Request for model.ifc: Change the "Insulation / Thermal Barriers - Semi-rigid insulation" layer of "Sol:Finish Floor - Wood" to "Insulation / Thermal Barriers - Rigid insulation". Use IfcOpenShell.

First a look at what the model holds.

```python
import ifcopenshell
import ifcopenshell.util.element

model = ifcopenshell.open("model.ifc")
print(model.schema)
for layer_set in model.by_type("IfcMaterialLayerSet"):
    if layer_set.LayerSetName == "Sol:Finish Floor - Wood":
        for layer in layer_set.MaterialLayers:
            print(layer.id(), layer.Material and layer.Material.Name, layer.LayerThickness, sep=" | ")
        print(len(ifcopenshell.util.element.get_elements_by_material(model, layer_set)), "elements and types use it")
print(sorted(m.Name for m in model.by_type("IfcMaterial") if m.Name)[:60])
```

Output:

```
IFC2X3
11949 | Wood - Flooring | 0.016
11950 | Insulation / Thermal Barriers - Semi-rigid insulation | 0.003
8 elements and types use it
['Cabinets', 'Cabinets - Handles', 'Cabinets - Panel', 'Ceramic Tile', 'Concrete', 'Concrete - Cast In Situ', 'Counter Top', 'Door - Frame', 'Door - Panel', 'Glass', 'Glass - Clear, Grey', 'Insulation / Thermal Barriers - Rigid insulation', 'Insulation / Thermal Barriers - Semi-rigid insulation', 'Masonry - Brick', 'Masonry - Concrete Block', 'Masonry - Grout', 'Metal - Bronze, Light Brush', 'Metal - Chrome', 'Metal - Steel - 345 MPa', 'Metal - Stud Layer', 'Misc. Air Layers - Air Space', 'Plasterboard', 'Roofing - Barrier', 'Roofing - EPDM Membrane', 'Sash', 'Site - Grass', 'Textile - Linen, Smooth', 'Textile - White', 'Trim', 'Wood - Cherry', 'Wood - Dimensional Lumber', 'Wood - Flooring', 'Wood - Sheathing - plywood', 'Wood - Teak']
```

```python
import ifcopenshell
import ifcopenshell.api.material

model = ifcopenshell.open("model.ifc")

layer_set = next(s for s in model.by_type("IfcMaterialLayerSet") if s.LayerSetName == "Sol:Finish Floor - Wood")
layer = next(l for l in layer_set.MaterialLayers if l.Material and l.Material.Name == "Insulation / Thermal Barriers - Semi-rigid insulation")
material = next(m for m in model.by_type("IfcMaterial") if m.Name == "Insulation / Thermal Barriers - Rigid insulation")

# Point this one layer at the other material; renaming the old one would change it everywhere.
ifcopenshell.api.material.edit_layer(model, layer=layer, attributes={}, material=material)

print([l.Material.Name if l.Material else None for l in layer_set.MaterialLayers])

model.write("model_rev.ifc")
```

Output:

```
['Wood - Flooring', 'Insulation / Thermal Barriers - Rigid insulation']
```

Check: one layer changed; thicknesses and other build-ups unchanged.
